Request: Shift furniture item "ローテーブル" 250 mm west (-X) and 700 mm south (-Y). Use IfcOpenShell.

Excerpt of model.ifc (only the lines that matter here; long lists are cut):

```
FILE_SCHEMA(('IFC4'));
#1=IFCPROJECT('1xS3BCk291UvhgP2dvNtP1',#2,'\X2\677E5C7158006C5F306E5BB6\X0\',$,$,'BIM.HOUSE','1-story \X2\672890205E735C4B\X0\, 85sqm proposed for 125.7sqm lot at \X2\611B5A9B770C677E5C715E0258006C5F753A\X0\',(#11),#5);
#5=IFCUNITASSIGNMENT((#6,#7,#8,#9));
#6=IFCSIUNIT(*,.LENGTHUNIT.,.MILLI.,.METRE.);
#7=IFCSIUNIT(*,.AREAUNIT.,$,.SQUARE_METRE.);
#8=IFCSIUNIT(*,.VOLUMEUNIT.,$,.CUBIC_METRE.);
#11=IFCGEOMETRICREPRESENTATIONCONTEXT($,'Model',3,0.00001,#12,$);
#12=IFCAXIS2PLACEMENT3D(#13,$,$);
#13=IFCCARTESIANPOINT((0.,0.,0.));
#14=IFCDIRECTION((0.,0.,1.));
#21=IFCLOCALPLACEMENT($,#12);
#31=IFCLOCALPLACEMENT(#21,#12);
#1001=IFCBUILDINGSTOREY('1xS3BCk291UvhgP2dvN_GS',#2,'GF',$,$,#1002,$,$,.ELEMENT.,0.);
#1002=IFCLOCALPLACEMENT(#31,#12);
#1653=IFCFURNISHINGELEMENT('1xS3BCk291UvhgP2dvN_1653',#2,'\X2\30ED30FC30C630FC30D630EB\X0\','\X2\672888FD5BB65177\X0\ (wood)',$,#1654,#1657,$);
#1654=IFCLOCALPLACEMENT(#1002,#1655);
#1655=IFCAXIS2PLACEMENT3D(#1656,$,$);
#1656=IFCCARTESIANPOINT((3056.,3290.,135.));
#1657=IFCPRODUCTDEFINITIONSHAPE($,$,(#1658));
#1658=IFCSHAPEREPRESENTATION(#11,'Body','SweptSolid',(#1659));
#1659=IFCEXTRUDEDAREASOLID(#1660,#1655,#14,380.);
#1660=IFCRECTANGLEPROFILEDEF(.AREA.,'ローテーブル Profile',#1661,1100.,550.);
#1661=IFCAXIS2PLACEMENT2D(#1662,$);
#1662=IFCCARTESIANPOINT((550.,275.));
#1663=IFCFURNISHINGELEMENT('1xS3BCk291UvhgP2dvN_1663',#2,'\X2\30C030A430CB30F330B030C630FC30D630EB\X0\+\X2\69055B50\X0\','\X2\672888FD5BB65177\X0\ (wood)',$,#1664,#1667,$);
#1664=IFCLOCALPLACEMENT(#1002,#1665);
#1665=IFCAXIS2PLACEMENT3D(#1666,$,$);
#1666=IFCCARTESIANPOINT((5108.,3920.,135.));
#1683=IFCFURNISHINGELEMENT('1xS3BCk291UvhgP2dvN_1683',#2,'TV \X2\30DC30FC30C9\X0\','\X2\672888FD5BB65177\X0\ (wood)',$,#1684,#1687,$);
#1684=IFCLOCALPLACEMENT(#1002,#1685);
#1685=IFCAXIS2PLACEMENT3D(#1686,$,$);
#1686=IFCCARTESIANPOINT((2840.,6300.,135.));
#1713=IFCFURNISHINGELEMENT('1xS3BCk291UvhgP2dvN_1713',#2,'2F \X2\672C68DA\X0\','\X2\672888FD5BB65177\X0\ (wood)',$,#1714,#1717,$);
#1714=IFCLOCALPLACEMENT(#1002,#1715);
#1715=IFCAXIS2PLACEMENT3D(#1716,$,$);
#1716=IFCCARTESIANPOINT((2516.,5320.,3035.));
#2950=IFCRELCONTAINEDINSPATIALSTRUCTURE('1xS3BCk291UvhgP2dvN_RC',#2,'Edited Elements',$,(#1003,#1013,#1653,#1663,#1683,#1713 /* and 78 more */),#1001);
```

```python
import ifcopenshell
import ifcopenshell.api.geometry
import ifcopenshell.util.placement
import ifcopenshell.util.unit

model = ifcopenshell.open("model.ifc")
unit_scale = ifcopenshell.util.unit.calculate_unit_scale(model)

item = model.by_id(1653)
matrix = ifcopenshell.util.placement.get_local_placement(item.ObjectPlacement)
matrix[0, 3] -= 0.25 / unit_scale
matrix[1, 3] -= 0.7 / unit_scale
ifcopenshell.api.geometry.edit_object_placement(model, product=item, matrix=matrix, is_si=False)

print(ifcopenshell.util.placement.get_local_placement(item.ObjectPlacement).round(3) + 0.0)

model.write("model_edited.ifc")
```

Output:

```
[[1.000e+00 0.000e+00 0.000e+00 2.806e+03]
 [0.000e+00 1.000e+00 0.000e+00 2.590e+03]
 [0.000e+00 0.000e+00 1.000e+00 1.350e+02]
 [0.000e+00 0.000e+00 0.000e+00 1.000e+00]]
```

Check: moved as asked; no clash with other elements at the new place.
